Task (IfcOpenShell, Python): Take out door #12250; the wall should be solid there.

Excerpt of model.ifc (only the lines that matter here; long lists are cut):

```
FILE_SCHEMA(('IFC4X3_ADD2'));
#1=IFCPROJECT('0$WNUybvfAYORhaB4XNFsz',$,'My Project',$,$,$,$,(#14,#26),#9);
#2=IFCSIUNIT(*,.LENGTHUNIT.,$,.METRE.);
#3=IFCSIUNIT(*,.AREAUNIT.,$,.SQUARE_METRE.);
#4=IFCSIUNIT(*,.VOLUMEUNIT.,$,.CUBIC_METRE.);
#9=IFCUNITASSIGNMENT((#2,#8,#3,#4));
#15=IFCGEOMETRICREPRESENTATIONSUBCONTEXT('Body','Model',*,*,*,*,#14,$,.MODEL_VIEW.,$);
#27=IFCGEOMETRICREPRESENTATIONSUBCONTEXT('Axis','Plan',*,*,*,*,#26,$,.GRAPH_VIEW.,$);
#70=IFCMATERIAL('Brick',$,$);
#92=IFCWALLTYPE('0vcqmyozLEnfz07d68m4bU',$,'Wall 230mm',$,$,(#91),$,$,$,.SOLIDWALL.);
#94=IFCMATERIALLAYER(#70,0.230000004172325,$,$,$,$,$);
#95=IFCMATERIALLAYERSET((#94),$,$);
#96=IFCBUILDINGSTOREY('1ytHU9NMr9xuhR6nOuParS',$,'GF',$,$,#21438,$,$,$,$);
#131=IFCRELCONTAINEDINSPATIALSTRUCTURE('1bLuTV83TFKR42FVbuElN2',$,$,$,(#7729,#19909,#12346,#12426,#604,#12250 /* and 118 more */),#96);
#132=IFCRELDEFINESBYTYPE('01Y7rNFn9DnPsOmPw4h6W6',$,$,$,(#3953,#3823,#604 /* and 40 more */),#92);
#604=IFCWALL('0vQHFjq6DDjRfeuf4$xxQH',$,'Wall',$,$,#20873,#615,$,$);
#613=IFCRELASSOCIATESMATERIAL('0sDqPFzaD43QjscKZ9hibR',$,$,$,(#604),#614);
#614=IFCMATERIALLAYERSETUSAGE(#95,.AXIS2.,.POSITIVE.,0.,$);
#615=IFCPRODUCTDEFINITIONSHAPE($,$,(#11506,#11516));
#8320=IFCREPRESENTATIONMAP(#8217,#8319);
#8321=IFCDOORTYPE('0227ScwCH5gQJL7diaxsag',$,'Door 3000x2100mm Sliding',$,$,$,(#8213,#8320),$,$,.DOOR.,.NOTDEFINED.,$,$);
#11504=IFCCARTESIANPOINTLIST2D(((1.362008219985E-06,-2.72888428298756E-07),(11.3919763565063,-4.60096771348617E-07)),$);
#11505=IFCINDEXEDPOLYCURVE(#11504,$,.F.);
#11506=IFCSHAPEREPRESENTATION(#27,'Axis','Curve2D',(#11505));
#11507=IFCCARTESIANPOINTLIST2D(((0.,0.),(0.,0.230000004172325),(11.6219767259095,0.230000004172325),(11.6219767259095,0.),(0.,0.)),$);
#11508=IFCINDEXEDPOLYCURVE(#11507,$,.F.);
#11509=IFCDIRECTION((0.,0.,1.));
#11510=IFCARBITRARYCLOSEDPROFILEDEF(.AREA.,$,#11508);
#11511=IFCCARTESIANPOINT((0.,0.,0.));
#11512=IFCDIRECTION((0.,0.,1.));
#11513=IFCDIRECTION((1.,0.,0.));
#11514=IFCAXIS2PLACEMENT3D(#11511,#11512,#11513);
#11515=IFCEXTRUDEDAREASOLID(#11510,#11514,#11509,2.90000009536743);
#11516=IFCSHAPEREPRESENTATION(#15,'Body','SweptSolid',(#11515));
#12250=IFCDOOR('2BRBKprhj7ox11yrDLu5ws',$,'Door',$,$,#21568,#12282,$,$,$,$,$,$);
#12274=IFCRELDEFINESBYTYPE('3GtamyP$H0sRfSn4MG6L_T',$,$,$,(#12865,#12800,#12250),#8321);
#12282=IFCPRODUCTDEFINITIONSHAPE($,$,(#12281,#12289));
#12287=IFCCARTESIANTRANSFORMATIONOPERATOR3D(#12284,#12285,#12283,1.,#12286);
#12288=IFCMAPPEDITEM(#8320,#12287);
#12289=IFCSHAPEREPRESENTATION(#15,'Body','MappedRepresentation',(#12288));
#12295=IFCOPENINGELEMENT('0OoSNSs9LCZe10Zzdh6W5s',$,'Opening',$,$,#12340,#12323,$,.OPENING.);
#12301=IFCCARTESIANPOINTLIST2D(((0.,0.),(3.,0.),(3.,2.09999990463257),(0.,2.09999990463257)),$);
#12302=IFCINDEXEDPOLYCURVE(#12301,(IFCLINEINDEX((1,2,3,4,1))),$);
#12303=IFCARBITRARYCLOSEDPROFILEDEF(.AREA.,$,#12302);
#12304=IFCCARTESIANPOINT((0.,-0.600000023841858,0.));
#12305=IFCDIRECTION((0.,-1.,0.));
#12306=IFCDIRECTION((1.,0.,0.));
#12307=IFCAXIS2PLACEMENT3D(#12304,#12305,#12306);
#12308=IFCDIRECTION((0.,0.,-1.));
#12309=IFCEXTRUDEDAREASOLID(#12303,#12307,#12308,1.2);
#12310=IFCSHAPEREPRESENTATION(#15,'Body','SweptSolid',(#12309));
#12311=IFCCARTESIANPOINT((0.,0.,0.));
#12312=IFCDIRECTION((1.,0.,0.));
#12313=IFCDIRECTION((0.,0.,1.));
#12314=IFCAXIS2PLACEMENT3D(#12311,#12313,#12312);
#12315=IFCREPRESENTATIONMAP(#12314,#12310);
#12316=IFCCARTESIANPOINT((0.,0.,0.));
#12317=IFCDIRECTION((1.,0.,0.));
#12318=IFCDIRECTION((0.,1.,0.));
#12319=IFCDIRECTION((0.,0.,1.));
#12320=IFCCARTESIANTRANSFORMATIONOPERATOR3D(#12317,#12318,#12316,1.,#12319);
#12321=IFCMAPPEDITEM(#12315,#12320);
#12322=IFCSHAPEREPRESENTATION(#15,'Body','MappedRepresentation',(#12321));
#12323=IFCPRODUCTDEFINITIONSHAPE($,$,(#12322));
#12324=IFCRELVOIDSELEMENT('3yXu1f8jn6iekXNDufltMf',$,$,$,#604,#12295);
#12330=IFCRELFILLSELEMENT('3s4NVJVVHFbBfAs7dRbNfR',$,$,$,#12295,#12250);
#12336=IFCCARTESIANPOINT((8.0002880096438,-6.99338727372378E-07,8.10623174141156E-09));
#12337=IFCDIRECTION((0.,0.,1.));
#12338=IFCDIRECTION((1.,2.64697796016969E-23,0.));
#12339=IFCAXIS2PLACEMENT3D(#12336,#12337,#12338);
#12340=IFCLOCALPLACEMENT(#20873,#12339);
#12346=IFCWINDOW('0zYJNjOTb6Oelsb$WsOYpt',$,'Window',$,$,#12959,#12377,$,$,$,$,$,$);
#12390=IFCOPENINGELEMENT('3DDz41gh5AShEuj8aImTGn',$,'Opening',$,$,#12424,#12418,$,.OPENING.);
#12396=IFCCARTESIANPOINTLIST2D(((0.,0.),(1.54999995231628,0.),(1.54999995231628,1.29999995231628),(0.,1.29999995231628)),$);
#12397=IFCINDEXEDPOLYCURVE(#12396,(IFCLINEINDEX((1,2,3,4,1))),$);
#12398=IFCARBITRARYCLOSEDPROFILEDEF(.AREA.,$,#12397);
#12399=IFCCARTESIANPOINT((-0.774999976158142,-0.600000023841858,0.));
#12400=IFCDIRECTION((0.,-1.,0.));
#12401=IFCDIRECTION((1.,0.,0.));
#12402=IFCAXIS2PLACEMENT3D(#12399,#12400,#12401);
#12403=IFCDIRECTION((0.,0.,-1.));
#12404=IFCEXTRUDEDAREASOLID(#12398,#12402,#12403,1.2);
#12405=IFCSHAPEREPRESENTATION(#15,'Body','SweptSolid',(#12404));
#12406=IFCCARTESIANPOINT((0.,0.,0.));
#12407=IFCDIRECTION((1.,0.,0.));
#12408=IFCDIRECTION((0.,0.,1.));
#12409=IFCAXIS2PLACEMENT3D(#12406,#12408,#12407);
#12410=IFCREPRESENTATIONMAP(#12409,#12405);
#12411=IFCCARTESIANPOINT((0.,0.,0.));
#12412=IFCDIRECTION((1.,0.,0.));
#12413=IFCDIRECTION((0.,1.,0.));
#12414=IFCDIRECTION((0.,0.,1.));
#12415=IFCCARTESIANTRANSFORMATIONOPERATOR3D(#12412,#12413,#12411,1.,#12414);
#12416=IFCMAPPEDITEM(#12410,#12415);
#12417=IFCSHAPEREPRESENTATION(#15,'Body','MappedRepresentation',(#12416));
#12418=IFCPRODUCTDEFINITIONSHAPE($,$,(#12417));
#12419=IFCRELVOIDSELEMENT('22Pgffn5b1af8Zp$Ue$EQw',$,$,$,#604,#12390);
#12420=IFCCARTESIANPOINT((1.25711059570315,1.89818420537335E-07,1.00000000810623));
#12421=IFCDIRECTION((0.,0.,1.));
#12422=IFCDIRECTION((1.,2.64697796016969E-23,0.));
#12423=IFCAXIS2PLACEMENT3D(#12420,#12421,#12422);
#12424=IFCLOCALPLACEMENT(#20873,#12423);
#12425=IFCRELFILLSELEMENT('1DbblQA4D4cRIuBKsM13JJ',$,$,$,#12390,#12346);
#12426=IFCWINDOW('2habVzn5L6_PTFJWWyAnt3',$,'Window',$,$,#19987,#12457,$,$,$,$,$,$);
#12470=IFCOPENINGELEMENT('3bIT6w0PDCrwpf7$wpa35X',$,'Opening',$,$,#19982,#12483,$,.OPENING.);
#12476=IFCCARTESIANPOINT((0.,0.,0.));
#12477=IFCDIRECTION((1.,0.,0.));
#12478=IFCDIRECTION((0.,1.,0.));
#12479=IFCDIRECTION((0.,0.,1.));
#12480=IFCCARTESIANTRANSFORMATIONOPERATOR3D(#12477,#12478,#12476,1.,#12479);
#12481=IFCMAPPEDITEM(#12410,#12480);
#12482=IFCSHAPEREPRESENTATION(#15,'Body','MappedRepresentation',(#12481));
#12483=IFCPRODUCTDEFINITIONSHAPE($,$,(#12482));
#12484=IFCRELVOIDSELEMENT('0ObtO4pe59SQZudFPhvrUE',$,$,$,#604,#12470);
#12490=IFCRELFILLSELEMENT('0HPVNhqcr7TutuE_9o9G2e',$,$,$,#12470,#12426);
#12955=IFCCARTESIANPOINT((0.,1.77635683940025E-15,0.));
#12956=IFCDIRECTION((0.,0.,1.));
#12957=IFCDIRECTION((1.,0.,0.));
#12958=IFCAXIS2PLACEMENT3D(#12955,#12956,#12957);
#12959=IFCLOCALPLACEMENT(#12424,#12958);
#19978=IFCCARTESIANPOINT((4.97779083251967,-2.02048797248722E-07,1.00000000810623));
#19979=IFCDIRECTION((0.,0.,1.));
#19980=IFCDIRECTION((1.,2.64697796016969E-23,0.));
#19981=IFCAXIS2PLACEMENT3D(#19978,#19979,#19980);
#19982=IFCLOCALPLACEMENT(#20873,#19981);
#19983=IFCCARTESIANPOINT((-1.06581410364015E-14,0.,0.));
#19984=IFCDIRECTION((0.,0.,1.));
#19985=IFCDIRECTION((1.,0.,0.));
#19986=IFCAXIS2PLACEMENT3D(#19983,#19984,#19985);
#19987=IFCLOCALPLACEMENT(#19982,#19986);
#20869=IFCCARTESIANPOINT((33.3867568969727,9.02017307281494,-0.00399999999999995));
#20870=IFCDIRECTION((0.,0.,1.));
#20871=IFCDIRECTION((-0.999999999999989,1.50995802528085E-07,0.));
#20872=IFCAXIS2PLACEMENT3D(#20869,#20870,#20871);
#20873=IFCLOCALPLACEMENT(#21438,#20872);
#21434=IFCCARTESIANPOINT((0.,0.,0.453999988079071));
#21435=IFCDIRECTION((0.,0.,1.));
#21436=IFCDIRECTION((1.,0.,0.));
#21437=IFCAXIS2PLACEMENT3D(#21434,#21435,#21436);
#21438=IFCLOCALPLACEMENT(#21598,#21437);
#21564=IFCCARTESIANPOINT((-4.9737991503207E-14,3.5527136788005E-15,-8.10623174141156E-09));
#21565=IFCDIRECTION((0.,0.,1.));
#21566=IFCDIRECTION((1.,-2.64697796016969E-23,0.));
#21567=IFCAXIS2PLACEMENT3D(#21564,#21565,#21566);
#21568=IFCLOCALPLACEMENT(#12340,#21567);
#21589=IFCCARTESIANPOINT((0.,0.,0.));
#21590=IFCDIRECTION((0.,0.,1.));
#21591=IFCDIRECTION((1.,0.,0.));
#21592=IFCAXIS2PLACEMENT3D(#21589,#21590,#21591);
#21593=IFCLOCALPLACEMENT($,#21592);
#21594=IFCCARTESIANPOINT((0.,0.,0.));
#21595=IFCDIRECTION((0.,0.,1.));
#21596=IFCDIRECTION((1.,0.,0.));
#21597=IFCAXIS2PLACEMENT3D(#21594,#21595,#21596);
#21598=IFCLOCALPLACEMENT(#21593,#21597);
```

```python
import ifcopenshell
import ifcopenshell.api.feature
import ifcopenshell.api.root
import ifcopenshell.geom
import ifcopenshell.util.shape

model = ifcopenshell.open("model.ifc")
settings = ifcopenshell.geom.settings()


def volume(element):
    """Net volume in cubic metres, openings subtracted."""
    shape = ifcopenshell.geom.create_shape(settings, element)
    return ifcopenshell.util.shape.get_volume(shape.geometry)


door = model.by_guid("2BRBKprhj7ox11yrDLu5ws")
opening = door.FillsVoids[0].RelatingOpeningElement
wall = opening.VoidsElements[0].RelatingBuildingElement
before = volume(wall)

ifcopenshell.api.root.remove_product(model, product=door)
ifcopenshell.api.feature.remove_feature(model, feature=opening)

after = volume(wall)

print(f"wall volume {before:.3f} -> {after:.3f} m3")

model.write("model_updated.ifc")
```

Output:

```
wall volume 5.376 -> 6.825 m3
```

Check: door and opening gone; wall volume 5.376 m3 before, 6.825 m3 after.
